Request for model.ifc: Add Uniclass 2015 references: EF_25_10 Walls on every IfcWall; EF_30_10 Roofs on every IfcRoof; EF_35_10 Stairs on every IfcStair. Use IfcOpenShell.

First a look at what the model holds.

```python
import ifcopenshell

model = ifcopenshell.open("model.ifc")
print(model.schema)
print("classifications:", [c.Name for c in model.by_type("IfcClassification")])
for ifc_class in ("IfcDoor", "IfcRoof", "IfcStair", "IfcWall", "IfcWindow"):
    print(ifc_class, len(model.by_type(ifc_class)))
```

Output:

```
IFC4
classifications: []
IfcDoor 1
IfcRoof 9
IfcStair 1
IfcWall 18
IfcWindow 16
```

```python
import ifcopenshell
import ifcopenshell.api.classification

model = ifcopenshell.open("model.ifc")

system = ifcopenshell.api.classification.add_classification(model, classification="Uniclass 2015")

codes = {
    "IfcWall": ("EF_25_10", "Walls"),
    "IfcRoof": ("EF_30_10", "Roofs"),
    "IfcStair": ("EF_35_10", "Stairs"),
}
for ifc_class, (code, name) in codes.items():
    products = model.by_type(ifc_class)
    ifcopenshell.api.classification.add_reference(
        model, products=products, classification=system, identification=code, name=name
    )
    print(code, len(products))

model.write("model_rev.ifc")
```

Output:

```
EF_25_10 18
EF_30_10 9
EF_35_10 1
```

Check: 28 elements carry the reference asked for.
